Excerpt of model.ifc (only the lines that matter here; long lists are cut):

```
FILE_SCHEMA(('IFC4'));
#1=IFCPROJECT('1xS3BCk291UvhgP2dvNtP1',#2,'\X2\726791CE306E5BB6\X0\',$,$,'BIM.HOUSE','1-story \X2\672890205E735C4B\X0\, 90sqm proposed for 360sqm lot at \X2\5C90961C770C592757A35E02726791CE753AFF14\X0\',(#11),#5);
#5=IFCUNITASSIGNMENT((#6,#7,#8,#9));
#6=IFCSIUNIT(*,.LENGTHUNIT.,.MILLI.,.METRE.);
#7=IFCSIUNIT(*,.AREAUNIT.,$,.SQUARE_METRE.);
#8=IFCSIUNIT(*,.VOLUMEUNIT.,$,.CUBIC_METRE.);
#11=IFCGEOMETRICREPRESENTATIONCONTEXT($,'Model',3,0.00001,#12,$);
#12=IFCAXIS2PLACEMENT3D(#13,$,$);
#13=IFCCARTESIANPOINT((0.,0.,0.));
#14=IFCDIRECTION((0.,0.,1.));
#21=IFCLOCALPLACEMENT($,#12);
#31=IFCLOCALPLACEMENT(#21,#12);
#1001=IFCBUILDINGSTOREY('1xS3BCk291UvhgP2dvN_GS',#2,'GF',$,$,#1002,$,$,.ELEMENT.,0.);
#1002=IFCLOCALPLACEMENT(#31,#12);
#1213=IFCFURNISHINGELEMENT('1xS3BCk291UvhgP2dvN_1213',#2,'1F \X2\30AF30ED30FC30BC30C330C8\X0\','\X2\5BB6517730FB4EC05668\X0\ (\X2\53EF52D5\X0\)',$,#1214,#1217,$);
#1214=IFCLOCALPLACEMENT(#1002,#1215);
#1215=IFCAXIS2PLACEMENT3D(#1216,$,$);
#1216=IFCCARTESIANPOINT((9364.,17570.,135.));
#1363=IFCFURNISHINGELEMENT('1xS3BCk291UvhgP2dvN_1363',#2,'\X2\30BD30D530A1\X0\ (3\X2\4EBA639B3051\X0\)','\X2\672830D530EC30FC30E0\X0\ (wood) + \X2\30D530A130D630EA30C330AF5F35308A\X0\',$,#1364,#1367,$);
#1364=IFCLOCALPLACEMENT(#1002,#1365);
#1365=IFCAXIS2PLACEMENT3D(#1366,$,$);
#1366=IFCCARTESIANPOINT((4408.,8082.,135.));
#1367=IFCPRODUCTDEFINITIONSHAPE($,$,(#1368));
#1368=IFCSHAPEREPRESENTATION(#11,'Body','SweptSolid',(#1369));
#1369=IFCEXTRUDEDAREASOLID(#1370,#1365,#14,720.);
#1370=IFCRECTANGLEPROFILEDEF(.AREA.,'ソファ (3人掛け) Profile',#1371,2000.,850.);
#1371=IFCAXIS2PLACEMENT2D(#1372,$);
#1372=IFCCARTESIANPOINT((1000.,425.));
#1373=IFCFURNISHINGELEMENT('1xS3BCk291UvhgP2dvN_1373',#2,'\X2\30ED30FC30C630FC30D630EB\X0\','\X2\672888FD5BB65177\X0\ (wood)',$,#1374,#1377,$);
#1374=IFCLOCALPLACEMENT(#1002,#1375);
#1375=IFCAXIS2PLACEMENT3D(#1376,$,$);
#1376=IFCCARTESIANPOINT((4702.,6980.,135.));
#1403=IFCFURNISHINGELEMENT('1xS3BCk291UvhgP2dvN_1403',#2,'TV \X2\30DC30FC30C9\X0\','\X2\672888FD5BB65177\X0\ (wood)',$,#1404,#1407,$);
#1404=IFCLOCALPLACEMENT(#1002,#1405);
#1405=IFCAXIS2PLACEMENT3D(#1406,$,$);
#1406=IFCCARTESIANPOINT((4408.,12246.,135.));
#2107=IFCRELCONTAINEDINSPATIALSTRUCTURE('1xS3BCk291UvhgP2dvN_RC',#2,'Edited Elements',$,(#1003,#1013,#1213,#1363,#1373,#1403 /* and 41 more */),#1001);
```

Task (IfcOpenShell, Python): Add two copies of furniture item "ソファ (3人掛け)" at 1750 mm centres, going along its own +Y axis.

```python
import ifcopenshell
import ifcopenshell.api.geometry
import ifcopenshell.api.root
import ifcopenshell.util.element
import ifcopenshell.util.placement

model = ifcopenshell.open("model.ifc")


def reuse_history(source, copy):
    """copy_class also copies each property set's owner history, people and application; keep the originals."""
    for rel in copy.IsDefinedBy:
        if rel.is_a("IfcRelDefinesByProperties") and (history := rel.RelatingPropertyDefinition.OwnerHistory):
            rel.RelatingPropertyDefinition.OwnerHistory = source.OwnerHistory
            ifcopenshell.util.element.remove_deep2(model, history)


source = model.by_id(1363)
base = ifcopenshell.util.placement.get_local_placement(source.ObjectPlacement)
step = base[:3, 1] * 1750.0

for i in range(1, 3):
    copy = ifcopenshell.api.root.copy_class(model, product=source)
    copy.Representation = ifcopenshell.util.element.copy_deep(
        model, source.Representation, exclude=["IfcGeometricRepresentationContext", "IfcRepresentationMap"]
    )
    reuse_history(source, copy)
    matrix = base.copy()
    matrix[:3, 3] += i * step
    print("added at", matrix[:3, 3].round(3) + 0.0)
    ifcopenshell.api.geometry.edit_object_placement(model, product=copy, matrix=matrix, is_si=False)

model.write("model_updated.ifc")
```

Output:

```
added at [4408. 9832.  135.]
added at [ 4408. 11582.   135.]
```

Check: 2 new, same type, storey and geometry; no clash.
